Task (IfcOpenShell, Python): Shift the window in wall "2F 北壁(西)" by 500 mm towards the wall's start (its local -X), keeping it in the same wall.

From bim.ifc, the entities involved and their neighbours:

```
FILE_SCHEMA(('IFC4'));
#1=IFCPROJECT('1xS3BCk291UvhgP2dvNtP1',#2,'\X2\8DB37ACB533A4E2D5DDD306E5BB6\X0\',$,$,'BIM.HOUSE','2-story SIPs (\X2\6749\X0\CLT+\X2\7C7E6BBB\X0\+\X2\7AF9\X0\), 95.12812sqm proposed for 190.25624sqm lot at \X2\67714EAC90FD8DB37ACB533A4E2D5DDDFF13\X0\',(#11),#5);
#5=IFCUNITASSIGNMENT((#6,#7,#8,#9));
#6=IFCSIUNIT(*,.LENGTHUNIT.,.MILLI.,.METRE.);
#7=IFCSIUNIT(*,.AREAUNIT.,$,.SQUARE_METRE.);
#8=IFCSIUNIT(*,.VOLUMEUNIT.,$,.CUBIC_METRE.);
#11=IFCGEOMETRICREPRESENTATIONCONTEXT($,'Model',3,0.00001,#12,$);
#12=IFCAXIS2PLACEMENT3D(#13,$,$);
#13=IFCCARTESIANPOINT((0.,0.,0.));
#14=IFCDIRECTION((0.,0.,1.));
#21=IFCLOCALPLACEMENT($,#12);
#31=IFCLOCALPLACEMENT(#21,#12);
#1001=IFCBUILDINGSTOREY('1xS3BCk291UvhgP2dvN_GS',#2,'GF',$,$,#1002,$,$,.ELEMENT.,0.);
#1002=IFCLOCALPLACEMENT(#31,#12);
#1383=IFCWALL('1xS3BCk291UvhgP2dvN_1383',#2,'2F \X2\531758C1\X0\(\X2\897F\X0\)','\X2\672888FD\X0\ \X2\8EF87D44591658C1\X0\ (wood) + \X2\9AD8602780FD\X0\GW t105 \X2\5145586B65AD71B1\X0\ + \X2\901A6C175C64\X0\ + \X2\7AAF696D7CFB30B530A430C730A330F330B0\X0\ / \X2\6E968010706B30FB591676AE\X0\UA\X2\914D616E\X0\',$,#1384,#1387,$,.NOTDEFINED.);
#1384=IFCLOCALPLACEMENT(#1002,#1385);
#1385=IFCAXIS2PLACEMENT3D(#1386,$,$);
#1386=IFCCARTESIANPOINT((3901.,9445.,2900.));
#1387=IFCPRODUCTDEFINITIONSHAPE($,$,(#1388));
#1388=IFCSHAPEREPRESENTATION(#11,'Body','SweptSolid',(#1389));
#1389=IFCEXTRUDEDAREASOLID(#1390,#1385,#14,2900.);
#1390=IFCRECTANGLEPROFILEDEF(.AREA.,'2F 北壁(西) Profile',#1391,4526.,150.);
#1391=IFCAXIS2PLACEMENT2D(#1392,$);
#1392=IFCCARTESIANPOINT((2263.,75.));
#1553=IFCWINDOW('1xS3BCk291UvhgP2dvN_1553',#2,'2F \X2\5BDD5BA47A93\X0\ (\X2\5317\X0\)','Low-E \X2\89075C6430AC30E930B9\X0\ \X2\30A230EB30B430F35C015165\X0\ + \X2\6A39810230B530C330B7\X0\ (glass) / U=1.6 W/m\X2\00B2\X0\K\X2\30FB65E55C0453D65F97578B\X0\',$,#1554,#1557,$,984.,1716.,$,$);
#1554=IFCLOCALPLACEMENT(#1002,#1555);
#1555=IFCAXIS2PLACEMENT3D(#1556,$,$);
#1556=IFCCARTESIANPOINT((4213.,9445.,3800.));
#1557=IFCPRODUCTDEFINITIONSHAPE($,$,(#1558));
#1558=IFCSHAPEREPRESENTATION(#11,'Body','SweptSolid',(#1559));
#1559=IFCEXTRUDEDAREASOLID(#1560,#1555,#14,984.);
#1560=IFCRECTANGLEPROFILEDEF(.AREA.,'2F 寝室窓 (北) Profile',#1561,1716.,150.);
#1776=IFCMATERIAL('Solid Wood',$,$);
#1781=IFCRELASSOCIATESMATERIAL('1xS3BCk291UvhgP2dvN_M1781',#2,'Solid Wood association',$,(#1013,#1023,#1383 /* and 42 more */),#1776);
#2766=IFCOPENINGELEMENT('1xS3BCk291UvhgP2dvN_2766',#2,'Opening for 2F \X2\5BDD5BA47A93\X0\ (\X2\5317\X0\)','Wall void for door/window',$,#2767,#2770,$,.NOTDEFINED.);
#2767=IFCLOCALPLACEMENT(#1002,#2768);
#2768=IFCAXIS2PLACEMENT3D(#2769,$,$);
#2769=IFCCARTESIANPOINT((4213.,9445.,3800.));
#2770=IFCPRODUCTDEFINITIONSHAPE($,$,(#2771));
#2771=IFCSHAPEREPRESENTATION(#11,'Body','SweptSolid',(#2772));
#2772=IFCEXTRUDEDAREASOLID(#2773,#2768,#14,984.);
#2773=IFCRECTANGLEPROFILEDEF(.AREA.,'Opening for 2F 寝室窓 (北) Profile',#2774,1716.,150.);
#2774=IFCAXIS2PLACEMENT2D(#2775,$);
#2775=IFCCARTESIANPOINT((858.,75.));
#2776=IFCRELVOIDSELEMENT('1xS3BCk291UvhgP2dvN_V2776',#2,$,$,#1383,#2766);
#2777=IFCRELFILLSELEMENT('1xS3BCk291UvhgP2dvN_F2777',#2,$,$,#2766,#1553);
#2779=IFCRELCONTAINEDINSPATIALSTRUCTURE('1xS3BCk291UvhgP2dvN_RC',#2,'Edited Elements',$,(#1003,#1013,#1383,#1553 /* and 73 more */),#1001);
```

```python
import ifcopenshell
import ifcopenshell.api.geometry
import ifcopenshell.util.placement

model = ifcopenshell.open("bim.ifc")

window = model.by_guid("1xS3BCk291UvhgP2dvN_1553")
opening = window.FillsVoids[0].RelatingOpeningElement
wall = opening.VoidsElements[0].RelatingBuildingElement

wall_matrix = ifcopenshell.util.placement.get_local_placement(wall.ObjectPlacement)
shift = wall_matrix[:3, 0] * -500.0
before = ifcopenshell.util.placement.get_local_placement(window.ObjectPlacement)[:3, 3].copy()

# The window is not placed relative to its opening, so move both.
for product in (opening, window):
    matrix = ifcopenshell.util.placement.get_local_placement(product.ObjectPlacement)
    matrix[:3, 3] += shift
    ifcopenshell.api.geometry.edit_object_placement(model, product=product, matrix=matrix, is_si=False)

after = ifcopenshell.util.placement.get_local_placement(window.ObjectPlacement)[:3, 3]
print("window moved by", (after - before).round(3) + 0.0)

model.write("bim_rev.ifc")
```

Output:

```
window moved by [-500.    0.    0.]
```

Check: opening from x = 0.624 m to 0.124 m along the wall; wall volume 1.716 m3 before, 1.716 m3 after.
